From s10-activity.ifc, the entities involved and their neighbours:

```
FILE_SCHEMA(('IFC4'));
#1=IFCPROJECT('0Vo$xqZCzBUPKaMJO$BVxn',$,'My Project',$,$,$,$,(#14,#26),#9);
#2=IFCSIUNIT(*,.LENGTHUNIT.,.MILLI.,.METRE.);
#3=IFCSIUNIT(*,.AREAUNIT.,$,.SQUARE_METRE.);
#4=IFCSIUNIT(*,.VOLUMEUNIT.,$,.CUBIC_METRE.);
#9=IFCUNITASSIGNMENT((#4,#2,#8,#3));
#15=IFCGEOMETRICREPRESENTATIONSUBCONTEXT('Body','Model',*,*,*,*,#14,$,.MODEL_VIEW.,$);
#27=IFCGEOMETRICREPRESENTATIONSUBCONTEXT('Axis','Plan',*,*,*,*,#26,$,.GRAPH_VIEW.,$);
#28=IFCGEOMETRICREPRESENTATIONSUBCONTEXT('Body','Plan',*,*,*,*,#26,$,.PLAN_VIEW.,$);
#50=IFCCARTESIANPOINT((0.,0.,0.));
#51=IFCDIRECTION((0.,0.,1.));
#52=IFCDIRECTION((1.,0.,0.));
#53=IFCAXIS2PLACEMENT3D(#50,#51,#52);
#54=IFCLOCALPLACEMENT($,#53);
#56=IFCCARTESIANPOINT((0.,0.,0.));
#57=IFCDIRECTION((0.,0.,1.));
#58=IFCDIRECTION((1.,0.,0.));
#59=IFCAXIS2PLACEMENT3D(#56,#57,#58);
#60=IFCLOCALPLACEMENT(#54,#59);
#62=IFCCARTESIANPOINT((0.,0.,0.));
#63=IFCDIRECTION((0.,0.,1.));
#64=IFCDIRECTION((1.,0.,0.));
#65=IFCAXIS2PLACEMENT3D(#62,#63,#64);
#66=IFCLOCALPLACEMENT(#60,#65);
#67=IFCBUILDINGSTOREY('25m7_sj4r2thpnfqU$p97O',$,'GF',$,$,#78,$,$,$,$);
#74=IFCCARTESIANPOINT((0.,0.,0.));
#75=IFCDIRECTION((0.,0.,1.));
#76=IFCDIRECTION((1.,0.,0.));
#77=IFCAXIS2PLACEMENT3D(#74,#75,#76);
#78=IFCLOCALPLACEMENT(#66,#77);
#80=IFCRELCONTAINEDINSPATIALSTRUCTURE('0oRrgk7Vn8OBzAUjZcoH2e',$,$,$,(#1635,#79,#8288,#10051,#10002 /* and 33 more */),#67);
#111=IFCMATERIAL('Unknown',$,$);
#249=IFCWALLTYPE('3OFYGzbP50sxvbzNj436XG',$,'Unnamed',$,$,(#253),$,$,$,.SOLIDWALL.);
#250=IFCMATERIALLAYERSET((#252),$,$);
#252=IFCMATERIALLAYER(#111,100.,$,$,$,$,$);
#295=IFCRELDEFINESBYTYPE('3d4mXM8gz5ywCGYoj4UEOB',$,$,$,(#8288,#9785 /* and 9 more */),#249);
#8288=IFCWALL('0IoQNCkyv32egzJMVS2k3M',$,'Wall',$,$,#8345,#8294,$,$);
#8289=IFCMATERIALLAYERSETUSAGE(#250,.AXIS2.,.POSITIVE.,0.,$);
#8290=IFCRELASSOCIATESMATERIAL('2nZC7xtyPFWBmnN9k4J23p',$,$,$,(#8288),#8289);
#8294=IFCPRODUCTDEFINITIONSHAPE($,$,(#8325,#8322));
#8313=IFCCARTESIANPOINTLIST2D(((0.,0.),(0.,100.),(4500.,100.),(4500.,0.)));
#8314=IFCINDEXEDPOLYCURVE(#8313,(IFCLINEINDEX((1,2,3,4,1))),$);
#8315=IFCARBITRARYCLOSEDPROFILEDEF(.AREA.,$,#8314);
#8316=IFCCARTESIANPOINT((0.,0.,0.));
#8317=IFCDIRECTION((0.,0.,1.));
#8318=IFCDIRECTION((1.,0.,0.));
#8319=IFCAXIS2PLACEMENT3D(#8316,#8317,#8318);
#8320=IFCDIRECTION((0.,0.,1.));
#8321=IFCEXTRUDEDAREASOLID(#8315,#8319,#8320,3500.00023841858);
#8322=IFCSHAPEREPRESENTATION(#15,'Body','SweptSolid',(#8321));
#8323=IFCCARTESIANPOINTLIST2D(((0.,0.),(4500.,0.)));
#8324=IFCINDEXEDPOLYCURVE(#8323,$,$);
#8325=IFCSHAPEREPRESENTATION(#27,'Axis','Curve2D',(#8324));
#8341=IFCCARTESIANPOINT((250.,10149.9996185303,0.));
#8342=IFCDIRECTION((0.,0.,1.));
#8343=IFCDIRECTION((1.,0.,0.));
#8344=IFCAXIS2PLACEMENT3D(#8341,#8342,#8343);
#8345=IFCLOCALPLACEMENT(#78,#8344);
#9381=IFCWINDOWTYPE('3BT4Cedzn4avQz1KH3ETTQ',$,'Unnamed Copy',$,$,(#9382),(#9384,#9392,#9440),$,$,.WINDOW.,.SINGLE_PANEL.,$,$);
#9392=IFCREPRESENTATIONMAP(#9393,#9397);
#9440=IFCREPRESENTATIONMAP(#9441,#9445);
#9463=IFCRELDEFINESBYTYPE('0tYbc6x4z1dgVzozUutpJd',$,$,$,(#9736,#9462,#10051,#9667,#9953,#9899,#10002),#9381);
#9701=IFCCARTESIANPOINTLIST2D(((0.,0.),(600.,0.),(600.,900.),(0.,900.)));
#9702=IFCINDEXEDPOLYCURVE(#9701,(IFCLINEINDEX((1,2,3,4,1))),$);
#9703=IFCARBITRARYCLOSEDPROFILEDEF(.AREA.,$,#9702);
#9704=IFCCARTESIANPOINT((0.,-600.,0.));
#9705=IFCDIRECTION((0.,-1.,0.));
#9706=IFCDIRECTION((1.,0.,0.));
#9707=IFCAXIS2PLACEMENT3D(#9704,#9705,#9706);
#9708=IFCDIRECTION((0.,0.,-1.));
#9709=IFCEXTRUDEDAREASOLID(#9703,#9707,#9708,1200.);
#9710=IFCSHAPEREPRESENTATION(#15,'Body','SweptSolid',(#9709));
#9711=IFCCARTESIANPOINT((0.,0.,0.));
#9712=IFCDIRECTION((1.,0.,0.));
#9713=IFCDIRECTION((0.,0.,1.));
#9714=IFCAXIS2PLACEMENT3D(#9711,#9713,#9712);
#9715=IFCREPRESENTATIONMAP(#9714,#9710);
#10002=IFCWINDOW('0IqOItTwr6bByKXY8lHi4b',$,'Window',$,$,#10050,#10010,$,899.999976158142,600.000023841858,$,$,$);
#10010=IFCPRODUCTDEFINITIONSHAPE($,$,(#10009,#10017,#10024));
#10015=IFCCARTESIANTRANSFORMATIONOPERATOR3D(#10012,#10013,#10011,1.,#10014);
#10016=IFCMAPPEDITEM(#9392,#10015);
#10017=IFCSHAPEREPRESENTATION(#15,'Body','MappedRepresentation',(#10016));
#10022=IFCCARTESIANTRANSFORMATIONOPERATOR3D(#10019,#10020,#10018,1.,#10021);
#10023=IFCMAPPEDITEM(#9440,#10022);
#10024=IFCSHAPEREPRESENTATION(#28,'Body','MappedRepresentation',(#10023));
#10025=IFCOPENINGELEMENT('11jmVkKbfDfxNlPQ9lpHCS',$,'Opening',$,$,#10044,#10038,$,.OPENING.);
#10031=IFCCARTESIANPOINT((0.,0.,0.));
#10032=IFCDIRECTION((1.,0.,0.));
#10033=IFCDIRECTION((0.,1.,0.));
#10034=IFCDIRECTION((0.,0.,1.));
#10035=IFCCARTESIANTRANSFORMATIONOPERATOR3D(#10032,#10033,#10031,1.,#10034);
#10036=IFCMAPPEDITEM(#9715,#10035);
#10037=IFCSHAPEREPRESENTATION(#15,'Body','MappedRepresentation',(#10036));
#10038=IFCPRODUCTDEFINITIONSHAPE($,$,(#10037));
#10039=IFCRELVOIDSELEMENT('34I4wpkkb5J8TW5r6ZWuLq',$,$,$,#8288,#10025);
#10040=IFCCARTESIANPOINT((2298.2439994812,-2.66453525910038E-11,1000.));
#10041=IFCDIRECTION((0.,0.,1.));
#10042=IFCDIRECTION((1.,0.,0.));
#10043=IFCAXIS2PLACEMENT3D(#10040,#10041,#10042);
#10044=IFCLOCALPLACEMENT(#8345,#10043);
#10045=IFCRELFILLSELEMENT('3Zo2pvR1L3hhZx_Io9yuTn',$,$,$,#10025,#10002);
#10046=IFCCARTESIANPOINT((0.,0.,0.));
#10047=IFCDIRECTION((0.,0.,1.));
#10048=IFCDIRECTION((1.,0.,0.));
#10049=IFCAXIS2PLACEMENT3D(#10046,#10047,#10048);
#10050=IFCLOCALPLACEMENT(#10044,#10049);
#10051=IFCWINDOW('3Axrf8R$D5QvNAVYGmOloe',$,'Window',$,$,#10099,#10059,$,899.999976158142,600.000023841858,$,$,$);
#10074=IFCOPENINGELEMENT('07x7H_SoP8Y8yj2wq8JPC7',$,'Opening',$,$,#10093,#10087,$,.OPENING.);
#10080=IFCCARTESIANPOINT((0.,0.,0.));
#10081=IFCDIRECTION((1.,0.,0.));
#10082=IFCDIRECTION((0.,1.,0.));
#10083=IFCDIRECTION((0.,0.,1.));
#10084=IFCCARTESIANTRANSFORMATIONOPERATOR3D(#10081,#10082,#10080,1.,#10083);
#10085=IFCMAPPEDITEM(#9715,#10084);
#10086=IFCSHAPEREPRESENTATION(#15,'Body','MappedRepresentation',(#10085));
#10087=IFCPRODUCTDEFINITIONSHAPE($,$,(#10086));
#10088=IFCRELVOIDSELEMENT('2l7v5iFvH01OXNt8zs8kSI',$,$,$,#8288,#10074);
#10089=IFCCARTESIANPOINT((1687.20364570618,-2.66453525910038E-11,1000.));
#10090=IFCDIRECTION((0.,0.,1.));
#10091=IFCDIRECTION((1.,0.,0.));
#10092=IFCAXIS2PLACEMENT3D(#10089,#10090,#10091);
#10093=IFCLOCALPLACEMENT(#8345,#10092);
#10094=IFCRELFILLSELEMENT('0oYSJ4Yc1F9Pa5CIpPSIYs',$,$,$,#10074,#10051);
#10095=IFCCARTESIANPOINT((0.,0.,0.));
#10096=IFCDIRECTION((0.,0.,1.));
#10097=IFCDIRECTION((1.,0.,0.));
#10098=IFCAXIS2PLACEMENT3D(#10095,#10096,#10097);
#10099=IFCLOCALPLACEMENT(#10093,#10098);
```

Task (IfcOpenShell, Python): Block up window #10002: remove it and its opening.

```python
import ifcopenshell
import ifcopenshell.api.feature
import ifcopenshell.api.root
import ifcopenshell.geom
import ifcopenshell.util.shape

model = ifcopenshell.open("s10-activity.ifc")
settings = ifcopenshell.geom.settings()


def volume(element):
    """Net volume in cubic metres, openings subtracted."""
    shape = ifcopenshell.geom.create_shape(settings, element)
    return ifcopenshell.util.shape.get_volume(shape.geometry)


window = model.by_guid("0IqOItTwr6bByKXY8lHi4b")
opening = window.FillsVoids[0].RelatingOpeningElement
wall = opening.VoidsElements[0].RelatingBuildingElement
before = volume(wall)

ifcopenshell.api.root.remove_product(model, product=window)
ifcopenshell.api.feature.remove_feature(model, feature=opening)

after = volume(wall)

print(f"wall volume {before:.3f} -> {after:.3f} m3")

model.write("s10-activity_rev.ifc")
```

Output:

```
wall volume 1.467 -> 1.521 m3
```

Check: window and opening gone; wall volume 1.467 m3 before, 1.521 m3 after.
